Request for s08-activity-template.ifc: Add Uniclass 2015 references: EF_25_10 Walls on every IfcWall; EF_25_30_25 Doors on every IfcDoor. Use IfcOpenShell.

First a look at what the model holds.

```python
import ifcopenshell

model = ifcopenshell.open("s08-activity-template.ifc")
print(model.schema)
print("classifications:", [c.Name for c in model.by_type("IfcClassification")])
for ifc_class in ("IfcDoor", "IfcRoof", "IfcStair", "IfcWall", "IfcWindow"):
    print(ifc_class, len(model.by_type(ifc_class)))
```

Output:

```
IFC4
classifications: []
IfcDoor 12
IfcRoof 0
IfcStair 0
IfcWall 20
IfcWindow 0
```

```python
import ifcopenshell
import ifcopenshell.api.classification

model = ifcopenshell.open("s08-activity-template.ifc")

system = ifcopenshell.api.classification.add_classification(model, classification="Uniclass 2015")

codes = {
    "IfcWall": ("EF_25_10", "Walls"),
    "IfcDoor": ("EF_25_30_25", "Doors"),
}
for ifc_class, (code, name) in codes.items():
    products = model.by_type(ifc_class)
    ifcopenshell.api.classification.add_reference(
        model, products=products, classification=system, identification=code, name=name
    )
    print(code, len(products))

model.write("s08-activity-template_updated.ifc")
```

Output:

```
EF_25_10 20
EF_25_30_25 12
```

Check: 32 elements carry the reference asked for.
